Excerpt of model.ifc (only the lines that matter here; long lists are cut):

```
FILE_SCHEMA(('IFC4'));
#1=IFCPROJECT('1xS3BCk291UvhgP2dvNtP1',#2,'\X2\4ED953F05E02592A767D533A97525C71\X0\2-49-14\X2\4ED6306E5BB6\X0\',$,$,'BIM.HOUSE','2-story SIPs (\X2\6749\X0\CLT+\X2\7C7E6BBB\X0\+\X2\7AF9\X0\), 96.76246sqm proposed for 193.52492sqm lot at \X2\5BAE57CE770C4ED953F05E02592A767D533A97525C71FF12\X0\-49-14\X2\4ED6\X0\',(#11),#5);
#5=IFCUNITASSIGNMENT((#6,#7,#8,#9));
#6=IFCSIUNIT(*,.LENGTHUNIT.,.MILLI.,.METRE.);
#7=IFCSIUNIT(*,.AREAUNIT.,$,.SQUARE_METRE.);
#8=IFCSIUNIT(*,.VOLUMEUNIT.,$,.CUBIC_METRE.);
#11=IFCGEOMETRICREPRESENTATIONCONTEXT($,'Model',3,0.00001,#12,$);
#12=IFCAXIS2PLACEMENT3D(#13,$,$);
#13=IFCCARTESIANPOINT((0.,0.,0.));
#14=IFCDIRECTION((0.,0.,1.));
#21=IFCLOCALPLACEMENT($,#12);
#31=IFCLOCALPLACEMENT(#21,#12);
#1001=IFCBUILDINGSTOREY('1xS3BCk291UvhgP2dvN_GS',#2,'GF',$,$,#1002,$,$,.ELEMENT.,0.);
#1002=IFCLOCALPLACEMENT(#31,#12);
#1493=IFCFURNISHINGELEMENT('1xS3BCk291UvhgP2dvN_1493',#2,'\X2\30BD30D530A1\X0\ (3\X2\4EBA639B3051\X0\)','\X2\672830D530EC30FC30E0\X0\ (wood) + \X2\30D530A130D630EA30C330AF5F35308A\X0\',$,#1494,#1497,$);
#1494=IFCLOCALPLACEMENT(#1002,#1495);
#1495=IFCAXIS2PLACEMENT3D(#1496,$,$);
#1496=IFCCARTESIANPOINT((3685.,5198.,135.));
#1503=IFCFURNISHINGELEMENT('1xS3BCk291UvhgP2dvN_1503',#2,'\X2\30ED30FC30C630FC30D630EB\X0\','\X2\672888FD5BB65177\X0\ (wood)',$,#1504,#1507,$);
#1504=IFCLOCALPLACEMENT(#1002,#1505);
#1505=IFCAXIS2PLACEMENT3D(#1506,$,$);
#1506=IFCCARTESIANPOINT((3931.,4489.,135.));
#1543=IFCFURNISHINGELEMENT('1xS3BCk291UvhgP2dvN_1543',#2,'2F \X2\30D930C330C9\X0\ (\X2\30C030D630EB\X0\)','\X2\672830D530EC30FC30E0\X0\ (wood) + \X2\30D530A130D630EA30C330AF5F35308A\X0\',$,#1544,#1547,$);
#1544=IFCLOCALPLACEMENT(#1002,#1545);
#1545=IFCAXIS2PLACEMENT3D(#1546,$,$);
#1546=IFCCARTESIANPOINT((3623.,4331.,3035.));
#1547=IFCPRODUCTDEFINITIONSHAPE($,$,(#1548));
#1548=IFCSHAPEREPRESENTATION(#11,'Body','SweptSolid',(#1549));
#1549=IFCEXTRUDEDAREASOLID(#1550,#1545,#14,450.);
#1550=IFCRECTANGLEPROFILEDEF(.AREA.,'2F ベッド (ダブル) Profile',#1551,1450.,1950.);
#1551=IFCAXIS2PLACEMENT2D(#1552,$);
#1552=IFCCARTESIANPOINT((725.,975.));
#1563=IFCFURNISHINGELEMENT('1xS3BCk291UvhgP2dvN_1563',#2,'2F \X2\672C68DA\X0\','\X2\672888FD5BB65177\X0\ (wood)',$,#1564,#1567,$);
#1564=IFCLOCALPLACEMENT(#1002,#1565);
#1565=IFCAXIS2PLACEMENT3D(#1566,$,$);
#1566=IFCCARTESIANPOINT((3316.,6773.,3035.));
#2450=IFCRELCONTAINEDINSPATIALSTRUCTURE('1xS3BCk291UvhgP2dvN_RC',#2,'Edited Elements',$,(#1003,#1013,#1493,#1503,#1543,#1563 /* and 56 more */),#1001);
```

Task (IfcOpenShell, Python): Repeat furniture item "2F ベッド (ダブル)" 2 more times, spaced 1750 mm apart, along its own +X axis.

```python
import ifcopenshell
import ifcopenshell.api.geometry
import ifcopenshell.api.root
import ifcopenshell.util.element
import ifcopenshell.util.placement
import ifcopenshell.util.unit

model = ifcopenshell.open("model.ifc")
unit_scale = ifcopenshell.util.unit.calculate_unit_scale(model)


def reuse_history(source, copy):
    """copy_class also copies each property set's owner history, people and application; keep the originals."""
    for rel in copy.IsDefinedBy:
        if rel.is_a("IfcRelDefinesByProperties") and (history := rel.RelatingPropertyDefinition.OwnerHistory):
            rel.RelatingPropertyDefinition.OwnerHistory = source.OwnerHistory
            ifcopenshell.util.element.remove_deep2(model, history)


source = model.by_guid("1xS3BCk291UvhgP2dvN_1543")
base = ifcopenshell.util.placement.get_local_placement(source.ObjectPlacement)
step = base[:3, 0] * 1.75 / unit_scale

for i in range(1, 3):
    copy = ifcopenshell.api.root.copy_class(model, product=source)
    copy.Representation = ifcopenshell.util.element.copy_deep(
        model, source.Representation, exclude=["IfcGeometricRepresentationContext", "IfcRepresentationMap"]
    )
    reuse_history(source, copy)
    matrix = base.copy()
    matrix[:3, 3] += i * step
    print("added at", matrix[:3, 3].round(3) + 0.0)
    ifcopenshell.api.geometry.edit_object_placement(model, product=copy, matrix=matrix, is_si=False)

model.write("model_edited.ifc")
```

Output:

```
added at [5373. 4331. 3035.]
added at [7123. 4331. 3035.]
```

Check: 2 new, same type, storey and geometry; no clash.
